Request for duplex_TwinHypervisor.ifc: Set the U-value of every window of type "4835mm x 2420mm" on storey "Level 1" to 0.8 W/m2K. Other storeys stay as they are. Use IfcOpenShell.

First a look at what the model holds.

```python
import ifcopenshell
import ifcopenshell.util.element

model = ifcopenshell.open("duplex_TwinHypervisor.ifc")
print(model.schema)
storey = next(s for s in model.by_type("IfcBuildingStorey") if s.Name == "Level 1")
windows = [e for e in ifcopenshell.util.element.get_decomposition(storey) if e.is_a("IfcWindow")]
seen = {}
for e in windows:
    element_type = ifcopenshell.util.element.get_type(e)
    key = (element_type.Name if element_type != e and element_type else None, ifcopenshell.util.element.get_pset(e, "Pset_WindowCommon", "ThermalTransmittance"))
    seen[key] = seen.get(key, 0) + 1
for (name, value), count in sorted(seen.items(), key=str):
    print(count, "x", name, "|", value)
```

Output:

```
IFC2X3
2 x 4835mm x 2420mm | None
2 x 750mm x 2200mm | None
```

```python
import ifcopenshell
import ifcopenshell.api.pset
import ifcopenshell.util.element

model = ifcopenshell.open("duplex_TwinHypervisor.ifc")

storey = next(s for s in model.by_type("IfcBuildingStorey") if s.Name == "Level 1")
windows = [e for e in ifcopenshell.util.element.get_decomposition(storey) if e.is_a("IfcWindow")]

count = 0
for e in windows:
    element_type = ifcopenshell.util.element.get_type(e)
    if element_type in (None, e) or element_type.Name != "4835mm x 2420mm":
        continue
    # add_pset returns the element's existing set when there is one.
    pset = ifcopenshell.api.pset.add_pset(model, product=e, name="Pset_WindowCommon")
    ifcopenshell.api.pset.edit_pset(model, pset=pset, properties={"ThermalTransmittance": 0.8})
    count += 1

print(count, "windows updated")

model.write("duplex_TwinHypervisor-out.ifc")
```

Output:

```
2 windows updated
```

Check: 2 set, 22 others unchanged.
